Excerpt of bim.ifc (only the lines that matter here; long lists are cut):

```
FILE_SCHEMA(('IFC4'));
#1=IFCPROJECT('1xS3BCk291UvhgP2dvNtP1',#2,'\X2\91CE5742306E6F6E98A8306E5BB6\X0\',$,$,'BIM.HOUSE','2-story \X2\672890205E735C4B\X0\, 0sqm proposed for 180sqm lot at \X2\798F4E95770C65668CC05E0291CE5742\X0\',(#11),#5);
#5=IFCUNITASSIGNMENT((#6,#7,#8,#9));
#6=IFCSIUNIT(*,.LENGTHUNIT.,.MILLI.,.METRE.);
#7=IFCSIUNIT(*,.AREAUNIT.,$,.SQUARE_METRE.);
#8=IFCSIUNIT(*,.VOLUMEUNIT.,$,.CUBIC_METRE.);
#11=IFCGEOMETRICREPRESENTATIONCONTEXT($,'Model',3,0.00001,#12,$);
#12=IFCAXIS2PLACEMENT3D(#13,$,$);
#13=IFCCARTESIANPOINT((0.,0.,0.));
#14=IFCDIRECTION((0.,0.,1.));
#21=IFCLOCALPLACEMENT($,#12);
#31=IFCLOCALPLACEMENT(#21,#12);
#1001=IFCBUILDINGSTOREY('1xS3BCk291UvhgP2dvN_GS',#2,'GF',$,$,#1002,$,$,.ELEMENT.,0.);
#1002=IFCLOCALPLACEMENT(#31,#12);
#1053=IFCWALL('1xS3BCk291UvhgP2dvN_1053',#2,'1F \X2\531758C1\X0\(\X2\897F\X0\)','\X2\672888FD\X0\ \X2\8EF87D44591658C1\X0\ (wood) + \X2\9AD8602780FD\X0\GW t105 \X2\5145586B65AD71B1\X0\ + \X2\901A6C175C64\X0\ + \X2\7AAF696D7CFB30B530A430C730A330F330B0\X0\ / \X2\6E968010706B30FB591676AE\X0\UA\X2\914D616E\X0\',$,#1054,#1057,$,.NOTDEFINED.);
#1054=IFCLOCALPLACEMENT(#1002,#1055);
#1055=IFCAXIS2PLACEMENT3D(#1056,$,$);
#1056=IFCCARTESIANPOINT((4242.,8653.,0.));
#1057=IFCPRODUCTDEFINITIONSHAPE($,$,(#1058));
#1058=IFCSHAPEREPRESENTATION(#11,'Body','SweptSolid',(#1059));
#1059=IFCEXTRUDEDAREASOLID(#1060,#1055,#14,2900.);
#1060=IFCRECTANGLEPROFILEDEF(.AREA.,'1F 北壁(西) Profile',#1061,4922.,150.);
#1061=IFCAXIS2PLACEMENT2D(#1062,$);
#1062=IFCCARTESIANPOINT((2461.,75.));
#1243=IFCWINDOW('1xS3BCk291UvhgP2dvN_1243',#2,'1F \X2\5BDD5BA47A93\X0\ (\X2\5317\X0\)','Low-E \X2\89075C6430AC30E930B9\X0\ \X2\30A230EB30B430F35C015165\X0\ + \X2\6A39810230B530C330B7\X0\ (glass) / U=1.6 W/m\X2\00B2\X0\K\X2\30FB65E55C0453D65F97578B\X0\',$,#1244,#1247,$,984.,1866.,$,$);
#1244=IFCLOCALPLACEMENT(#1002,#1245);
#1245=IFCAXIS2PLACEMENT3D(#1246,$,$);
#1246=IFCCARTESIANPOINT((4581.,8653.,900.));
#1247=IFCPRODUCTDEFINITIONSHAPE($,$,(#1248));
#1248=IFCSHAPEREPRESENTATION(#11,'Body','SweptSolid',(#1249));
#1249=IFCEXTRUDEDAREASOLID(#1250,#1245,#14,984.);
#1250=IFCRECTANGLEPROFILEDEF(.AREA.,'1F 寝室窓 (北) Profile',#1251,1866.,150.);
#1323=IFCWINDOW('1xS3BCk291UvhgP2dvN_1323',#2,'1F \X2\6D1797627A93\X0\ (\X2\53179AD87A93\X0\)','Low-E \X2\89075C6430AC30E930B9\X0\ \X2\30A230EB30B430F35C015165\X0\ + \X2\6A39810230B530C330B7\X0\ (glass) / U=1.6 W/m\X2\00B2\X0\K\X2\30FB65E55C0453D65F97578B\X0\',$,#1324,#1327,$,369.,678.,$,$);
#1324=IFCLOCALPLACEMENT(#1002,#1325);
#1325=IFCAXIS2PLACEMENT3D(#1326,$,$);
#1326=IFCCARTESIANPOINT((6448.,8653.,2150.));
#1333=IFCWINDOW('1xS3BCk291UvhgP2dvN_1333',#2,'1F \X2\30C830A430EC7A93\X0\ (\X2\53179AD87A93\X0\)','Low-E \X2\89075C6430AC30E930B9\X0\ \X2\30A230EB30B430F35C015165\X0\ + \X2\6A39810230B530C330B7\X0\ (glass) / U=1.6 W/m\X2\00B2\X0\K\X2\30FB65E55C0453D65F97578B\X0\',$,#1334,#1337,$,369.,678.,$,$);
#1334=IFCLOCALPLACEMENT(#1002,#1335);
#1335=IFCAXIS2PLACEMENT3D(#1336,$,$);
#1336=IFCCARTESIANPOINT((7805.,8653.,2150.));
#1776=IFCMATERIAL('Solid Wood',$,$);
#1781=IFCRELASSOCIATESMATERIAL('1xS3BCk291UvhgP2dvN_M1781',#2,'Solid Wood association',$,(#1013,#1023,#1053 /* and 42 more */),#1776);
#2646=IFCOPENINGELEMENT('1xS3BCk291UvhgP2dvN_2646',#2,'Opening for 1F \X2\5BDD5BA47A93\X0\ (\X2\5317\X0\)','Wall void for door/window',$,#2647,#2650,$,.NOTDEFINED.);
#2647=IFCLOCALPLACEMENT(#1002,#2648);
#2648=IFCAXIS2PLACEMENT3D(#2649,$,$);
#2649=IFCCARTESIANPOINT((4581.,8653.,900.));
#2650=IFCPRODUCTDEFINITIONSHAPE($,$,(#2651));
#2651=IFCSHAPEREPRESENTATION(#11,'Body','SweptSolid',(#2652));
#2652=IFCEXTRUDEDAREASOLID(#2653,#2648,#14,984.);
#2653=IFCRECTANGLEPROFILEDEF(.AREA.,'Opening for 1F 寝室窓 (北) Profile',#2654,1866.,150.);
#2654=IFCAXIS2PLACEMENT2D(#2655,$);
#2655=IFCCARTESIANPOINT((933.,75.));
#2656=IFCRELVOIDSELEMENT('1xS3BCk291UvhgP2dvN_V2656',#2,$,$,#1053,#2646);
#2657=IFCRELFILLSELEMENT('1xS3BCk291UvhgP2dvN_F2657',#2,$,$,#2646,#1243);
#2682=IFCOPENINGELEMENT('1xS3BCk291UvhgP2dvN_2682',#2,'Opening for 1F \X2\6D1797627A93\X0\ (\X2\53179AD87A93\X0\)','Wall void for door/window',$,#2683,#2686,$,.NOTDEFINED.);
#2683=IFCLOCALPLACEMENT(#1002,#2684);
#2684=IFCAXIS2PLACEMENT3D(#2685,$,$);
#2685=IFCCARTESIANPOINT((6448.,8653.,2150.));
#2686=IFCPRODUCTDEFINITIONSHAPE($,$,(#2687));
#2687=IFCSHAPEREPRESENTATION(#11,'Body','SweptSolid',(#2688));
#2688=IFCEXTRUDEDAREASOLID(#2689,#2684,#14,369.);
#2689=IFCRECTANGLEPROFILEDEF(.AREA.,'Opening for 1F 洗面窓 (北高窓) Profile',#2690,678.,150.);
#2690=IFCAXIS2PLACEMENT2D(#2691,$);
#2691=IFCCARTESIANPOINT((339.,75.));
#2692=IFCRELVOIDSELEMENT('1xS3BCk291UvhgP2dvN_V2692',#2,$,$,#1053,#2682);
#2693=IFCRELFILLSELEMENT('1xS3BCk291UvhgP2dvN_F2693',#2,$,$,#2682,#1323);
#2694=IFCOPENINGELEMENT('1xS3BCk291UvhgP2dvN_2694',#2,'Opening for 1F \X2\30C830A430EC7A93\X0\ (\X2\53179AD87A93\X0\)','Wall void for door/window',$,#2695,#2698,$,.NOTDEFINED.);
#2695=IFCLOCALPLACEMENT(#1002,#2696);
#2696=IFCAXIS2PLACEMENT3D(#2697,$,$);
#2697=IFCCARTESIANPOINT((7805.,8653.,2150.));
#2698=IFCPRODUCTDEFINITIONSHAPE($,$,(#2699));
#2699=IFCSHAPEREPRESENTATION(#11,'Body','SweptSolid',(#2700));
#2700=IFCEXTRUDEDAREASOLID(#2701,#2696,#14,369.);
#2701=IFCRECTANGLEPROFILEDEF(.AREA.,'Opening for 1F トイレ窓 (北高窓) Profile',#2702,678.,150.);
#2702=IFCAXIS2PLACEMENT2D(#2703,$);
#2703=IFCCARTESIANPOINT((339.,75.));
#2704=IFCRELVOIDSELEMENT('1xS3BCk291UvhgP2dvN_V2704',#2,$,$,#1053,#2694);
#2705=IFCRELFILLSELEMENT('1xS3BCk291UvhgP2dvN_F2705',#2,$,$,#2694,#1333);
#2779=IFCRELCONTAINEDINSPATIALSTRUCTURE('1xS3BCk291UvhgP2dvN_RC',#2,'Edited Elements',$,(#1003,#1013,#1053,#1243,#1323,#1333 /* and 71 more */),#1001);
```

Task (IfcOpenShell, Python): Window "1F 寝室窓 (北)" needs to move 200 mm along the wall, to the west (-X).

```python
import ifcopenshell
import ifcopenshell.api.geometry
import ifcopenshell.util.placement
import ifcopenshell.util.unit

model = ifcopenshell.open("bim.ifc")
unit_scale = ifcopenshell.util.unit.calculate_unit_scale(model)

window = model.by_guid("1xS3BCk291UvhgP2dvN_1243")
opening = window.FillsVoids[0].RelatingOpeningElement
wall = opening.VoidsElements[0].RelatingBuildingElement

wall_matrix = ifcopenshell.util.placement.get_local_placement(wall.ObjectPlacement)
shift = wall_matrix[:3, 0] * -0.2 / unit_scale
before = ifcopenshell.util.placement.get_local_placement(window.ObjectPlacement)[:3, 3].copy()

# The window is not placed relative to its opening, so move both.
for product in (opening, window):
    matrix = ifcopenshell.util.placement.get_local_placement(product.ObjectPlacement)
    matrix[:3, 3] += shift
    ifcopenshell.api.geometry.edit_object_placement(model, product=product, matrix=matrix, is_si=False)

after = ifcopenshell.util.placement.get_local_placement(window.ObjectPlacement)[:3, 3]
print("window moved by", (after - before).round(3) + 0.0)

model.write("bim-out.ifc")
```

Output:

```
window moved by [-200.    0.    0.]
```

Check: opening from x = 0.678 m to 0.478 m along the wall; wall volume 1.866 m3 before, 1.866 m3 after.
